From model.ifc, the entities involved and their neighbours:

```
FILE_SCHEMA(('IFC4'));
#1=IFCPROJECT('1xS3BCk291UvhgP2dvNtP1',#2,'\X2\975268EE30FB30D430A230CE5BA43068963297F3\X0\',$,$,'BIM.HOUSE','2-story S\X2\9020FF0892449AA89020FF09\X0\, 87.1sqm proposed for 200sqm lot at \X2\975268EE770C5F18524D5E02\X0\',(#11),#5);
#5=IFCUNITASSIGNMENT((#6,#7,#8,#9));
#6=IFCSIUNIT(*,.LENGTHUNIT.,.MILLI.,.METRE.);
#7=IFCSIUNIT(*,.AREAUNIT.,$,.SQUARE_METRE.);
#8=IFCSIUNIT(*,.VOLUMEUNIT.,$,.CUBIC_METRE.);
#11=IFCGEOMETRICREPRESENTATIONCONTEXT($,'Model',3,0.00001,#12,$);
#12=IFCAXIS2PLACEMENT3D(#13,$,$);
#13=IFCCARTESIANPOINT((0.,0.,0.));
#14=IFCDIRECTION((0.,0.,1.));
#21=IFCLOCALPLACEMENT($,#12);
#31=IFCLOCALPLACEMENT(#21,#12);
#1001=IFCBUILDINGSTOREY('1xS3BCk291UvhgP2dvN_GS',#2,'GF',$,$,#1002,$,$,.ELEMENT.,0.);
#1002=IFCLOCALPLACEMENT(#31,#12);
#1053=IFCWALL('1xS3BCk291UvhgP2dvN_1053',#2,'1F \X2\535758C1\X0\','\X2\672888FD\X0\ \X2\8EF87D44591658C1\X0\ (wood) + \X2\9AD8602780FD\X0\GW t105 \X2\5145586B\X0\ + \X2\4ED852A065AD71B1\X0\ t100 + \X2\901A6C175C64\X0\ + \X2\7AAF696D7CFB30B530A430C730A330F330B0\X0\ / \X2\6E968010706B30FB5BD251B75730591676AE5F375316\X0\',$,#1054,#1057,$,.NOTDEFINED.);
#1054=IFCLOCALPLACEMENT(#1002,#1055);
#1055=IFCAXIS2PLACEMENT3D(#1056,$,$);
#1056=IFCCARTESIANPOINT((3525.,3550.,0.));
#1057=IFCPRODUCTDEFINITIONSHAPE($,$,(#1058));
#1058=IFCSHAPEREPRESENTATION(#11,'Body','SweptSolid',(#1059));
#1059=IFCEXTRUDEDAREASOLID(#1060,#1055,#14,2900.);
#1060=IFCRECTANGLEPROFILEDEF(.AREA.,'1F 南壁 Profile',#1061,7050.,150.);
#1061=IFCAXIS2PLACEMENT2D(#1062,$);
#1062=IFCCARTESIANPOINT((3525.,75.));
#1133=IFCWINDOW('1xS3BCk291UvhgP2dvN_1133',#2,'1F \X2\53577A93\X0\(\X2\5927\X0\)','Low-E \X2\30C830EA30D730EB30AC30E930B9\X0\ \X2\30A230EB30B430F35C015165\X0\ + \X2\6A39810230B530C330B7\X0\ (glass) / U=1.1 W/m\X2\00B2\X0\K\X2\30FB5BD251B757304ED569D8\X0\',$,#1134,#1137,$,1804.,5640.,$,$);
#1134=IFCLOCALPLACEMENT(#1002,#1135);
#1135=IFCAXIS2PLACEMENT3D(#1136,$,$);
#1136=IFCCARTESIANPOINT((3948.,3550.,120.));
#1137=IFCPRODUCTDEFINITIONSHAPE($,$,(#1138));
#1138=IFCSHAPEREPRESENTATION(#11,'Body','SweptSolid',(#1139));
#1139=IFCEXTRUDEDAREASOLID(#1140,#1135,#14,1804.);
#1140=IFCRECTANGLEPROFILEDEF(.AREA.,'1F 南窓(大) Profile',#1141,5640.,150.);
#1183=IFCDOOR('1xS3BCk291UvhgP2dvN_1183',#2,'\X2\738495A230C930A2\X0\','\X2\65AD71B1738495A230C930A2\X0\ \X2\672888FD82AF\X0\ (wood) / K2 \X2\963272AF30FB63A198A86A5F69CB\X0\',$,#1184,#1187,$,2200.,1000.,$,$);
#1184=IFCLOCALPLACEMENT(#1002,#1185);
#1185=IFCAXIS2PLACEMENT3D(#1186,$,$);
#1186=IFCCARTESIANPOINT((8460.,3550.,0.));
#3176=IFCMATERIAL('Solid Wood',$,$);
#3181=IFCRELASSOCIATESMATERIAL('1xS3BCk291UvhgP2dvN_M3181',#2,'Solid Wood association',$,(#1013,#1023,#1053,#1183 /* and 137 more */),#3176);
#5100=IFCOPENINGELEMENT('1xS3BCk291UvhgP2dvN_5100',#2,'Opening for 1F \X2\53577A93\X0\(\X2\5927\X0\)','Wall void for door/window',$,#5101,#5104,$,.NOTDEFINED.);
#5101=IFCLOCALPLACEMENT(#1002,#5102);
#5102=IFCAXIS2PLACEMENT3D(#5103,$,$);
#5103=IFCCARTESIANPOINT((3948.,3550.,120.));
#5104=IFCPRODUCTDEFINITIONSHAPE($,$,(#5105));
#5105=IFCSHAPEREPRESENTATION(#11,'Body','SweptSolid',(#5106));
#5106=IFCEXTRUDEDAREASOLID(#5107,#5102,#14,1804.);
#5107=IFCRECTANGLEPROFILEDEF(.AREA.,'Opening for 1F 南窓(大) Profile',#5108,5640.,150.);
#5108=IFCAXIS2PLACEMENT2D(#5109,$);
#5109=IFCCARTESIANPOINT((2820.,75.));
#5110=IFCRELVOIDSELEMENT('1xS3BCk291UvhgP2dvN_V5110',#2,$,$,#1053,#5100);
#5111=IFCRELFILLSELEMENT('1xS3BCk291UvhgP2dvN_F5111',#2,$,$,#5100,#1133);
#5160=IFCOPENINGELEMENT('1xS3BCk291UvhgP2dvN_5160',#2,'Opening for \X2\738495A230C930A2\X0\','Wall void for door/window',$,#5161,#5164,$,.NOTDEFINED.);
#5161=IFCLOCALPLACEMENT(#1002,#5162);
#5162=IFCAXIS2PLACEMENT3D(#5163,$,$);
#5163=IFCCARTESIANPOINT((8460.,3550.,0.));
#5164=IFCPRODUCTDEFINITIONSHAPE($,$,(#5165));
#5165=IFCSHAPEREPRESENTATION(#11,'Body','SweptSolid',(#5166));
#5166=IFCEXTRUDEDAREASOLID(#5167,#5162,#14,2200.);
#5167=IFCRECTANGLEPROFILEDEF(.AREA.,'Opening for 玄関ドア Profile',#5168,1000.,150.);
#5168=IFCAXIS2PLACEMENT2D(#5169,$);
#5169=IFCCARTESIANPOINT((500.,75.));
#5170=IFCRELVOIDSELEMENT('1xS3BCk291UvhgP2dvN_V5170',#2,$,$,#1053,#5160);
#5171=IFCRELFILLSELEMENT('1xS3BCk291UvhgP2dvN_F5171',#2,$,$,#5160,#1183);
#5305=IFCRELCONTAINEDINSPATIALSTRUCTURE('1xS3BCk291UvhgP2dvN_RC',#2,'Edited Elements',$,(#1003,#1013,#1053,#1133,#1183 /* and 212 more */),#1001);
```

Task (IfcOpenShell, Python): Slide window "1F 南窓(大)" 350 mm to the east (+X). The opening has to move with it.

```python
import ifcopenshell
import ifcopenshell.api.geometry
import ifcopenshell.util.placement
import ifcopenshell.util.unit

model = ifcopenshell.open("model.ifc")
unit_scale = ifcopenshell.util.unit.calculate_unit_scale(model)

window = model.by_guid("1xS3BCk291UvhgP2dvN_1133")
opening = window.FillsVoids[0].RelatingOpeningElement
wall = opening.VoidsElements[0].RelatingBuildingElement

wall_matrix = ifcopenshell.util.placement.get_local_placement(wall.ObjectPlacement)
shift = wall_matrix[:3, 0] * 0.35 / unit_scale
before = ifcopenshell.util.placement.get_local_placement(window.ObjectPlacement)[:3, 3].copy()

# The window is not placed relative to its opening, so move both.
for product in (opening, window):
    matrix = ifcopenshell.util.placement.get_local_placement(product.ObjectPlacement)
    matrix[:3, 3] += shift
    ifcopenshell.api.geometry.edit_object_placement(model, product=product, matrix=matrix, is_si=False)

after = ifcopenshell.util.placement.get_local_placement(window.ObjectPlacement)[:3, 3]
print("window moved by", (after - before).round(3) + 0.0)

model.write("model-out.ifc")
```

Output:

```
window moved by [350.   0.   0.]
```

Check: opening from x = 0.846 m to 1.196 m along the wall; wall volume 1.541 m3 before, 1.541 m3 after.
